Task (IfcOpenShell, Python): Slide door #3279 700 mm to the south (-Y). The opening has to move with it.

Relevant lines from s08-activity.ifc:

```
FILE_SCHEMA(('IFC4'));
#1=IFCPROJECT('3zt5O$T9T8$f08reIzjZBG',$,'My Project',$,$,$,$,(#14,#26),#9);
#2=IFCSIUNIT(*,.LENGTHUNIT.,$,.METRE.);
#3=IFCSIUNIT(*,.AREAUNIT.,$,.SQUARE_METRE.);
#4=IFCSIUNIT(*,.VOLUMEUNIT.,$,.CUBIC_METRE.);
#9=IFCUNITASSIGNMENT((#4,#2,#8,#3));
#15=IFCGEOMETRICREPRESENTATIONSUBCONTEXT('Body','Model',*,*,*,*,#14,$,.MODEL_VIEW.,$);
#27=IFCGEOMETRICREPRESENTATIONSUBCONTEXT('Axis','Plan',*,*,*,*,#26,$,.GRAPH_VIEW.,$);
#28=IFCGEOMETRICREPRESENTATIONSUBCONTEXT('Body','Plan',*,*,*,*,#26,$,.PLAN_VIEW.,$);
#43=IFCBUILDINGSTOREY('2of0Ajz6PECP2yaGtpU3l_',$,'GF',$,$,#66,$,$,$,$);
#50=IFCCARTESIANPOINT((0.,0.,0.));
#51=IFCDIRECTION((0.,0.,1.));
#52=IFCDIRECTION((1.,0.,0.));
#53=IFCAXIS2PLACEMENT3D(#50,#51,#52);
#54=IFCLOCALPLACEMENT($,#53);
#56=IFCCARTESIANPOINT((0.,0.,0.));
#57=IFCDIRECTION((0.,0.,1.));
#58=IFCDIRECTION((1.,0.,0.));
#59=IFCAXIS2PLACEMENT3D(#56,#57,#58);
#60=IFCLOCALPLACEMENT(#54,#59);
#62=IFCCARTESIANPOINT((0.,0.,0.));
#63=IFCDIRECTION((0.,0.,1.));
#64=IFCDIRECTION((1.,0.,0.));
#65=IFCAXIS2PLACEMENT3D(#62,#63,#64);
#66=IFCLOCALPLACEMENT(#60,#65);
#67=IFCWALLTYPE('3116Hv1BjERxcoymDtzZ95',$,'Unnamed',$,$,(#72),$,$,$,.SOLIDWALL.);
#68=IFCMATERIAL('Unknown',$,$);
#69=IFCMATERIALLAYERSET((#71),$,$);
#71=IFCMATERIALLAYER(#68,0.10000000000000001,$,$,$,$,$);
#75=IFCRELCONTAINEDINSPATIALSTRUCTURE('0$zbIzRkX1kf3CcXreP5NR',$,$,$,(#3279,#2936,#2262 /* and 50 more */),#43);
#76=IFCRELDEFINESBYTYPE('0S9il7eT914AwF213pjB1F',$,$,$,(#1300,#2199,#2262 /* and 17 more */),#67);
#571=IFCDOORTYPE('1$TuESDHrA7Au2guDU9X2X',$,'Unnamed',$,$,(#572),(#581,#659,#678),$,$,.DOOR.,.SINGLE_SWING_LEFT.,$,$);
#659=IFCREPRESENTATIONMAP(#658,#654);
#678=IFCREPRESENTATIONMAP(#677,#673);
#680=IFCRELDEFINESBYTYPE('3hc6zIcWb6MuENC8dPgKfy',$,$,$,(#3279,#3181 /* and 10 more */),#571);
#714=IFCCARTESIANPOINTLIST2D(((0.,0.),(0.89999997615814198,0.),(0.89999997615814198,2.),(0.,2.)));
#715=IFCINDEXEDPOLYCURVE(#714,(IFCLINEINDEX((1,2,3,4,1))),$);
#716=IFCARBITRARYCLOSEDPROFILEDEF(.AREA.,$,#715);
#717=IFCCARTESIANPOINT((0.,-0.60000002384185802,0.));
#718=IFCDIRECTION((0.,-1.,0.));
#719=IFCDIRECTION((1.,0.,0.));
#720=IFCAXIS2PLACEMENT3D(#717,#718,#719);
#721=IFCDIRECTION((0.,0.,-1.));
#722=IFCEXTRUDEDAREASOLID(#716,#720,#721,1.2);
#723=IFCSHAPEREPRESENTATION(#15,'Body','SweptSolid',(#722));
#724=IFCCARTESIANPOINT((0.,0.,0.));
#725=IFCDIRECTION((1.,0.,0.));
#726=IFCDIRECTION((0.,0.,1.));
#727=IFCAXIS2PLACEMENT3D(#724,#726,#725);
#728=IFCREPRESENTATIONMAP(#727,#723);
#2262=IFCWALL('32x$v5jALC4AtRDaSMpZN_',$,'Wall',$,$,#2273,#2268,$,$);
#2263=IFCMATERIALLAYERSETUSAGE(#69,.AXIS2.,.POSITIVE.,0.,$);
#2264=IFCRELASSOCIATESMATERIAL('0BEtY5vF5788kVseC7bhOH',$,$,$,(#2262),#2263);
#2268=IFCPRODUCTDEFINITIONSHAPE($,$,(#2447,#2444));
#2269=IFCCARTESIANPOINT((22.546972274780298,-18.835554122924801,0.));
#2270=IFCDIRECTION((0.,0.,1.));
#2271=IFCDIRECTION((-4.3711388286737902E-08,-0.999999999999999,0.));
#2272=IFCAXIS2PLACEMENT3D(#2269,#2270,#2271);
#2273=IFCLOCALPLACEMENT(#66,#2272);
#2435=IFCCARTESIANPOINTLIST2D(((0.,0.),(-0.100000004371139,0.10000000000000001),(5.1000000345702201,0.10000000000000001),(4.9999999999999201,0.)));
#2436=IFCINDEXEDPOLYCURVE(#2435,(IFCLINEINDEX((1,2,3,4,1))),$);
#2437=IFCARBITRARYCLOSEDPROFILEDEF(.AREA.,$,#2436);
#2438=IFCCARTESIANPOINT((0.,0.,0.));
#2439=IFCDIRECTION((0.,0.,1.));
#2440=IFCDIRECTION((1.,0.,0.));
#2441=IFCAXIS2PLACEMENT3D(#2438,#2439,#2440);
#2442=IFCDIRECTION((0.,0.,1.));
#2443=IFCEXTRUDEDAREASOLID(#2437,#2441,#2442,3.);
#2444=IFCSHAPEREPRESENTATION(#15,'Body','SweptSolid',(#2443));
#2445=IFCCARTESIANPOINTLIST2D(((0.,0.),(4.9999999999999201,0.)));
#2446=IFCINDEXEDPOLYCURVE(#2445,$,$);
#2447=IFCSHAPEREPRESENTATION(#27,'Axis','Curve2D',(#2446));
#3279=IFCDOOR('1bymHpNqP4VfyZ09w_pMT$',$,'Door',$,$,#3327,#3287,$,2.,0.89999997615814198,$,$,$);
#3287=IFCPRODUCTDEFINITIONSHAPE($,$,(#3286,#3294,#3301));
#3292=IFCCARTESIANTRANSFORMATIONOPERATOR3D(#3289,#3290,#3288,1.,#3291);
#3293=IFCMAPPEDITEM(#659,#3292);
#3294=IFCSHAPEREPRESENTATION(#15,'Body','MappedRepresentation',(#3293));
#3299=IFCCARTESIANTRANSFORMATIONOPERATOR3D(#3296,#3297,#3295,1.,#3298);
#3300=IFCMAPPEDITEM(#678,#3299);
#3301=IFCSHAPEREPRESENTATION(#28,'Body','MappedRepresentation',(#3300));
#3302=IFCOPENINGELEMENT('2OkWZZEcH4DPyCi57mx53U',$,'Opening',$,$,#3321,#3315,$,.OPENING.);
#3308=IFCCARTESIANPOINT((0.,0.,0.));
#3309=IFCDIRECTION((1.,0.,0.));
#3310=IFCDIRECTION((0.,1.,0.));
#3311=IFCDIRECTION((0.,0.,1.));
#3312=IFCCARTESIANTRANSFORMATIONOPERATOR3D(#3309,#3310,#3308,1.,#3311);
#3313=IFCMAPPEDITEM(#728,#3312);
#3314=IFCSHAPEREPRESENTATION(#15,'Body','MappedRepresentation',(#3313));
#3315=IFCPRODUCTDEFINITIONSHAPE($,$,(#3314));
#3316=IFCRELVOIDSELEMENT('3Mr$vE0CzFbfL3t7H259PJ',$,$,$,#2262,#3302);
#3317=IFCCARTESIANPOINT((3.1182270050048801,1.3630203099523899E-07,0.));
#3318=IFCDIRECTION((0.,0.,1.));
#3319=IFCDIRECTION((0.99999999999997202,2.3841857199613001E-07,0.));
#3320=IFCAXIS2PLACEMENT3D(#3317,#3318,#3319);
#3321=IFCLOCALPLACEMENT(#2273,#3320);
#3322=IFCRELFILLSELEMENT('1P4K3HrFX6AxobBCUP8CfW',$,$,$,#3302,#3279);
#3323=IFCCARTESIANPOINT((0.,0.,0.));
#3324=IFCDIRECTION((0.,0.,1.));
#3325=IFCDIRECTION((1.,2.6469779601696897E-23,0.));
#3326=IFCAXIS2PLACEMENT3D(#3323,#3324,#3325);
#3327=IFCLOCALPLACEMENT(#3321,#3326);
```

```python
import ifcopenshell
import ifcopenshell.api.geometry
import ifcopenshell.util.placement
import ifcopenshell.util.unit

model = ifcopenshell.open("s08-activity.ifc")
unit_scale = ifcopenshell.util.unit.calculate_unit_scale(model)

door = model.by_guid("1bymHpNqP4VfyZ09w_pMT$")
opening = door.FillsVoids[0].RelatingOpeningElement
wall = opening.VoidsElements[0].RelatingBuildingElement

wall_matrix = ifcopenshell.util.placement.get_local_placement(wall.ObjectPlacement)
shift = wall_matrix[:3, 0] * 0.7 / unit_scale
before = ifcopenshell.util.placement.get_local_placement(door.ObjectPlacement)[:3, 3].copy()

# The door is placed relative to its opening, so it follows when the opening moves.
matrix = ifcopenshell.util.placement.get_local_placement(opening.ObjectPlacement)
matrix[:3, 3] += shift
ifcopenshell.api.geometry.edit_object_placement(
    model, product=opening, matrix=matrix, is_si=False, should_transform_children=True
)

after = ifcopenshell.util.placement.get_local_placement(door.ObjectPlacement)[:3, 3]
print("door moved by", (after - before).round(3) + 0.0)

model.write("s08-activity_v2.ifc")
```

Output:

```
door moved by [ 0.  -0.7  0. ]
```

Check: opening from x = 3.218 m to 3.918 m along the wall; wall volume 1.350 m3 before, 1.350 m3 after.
